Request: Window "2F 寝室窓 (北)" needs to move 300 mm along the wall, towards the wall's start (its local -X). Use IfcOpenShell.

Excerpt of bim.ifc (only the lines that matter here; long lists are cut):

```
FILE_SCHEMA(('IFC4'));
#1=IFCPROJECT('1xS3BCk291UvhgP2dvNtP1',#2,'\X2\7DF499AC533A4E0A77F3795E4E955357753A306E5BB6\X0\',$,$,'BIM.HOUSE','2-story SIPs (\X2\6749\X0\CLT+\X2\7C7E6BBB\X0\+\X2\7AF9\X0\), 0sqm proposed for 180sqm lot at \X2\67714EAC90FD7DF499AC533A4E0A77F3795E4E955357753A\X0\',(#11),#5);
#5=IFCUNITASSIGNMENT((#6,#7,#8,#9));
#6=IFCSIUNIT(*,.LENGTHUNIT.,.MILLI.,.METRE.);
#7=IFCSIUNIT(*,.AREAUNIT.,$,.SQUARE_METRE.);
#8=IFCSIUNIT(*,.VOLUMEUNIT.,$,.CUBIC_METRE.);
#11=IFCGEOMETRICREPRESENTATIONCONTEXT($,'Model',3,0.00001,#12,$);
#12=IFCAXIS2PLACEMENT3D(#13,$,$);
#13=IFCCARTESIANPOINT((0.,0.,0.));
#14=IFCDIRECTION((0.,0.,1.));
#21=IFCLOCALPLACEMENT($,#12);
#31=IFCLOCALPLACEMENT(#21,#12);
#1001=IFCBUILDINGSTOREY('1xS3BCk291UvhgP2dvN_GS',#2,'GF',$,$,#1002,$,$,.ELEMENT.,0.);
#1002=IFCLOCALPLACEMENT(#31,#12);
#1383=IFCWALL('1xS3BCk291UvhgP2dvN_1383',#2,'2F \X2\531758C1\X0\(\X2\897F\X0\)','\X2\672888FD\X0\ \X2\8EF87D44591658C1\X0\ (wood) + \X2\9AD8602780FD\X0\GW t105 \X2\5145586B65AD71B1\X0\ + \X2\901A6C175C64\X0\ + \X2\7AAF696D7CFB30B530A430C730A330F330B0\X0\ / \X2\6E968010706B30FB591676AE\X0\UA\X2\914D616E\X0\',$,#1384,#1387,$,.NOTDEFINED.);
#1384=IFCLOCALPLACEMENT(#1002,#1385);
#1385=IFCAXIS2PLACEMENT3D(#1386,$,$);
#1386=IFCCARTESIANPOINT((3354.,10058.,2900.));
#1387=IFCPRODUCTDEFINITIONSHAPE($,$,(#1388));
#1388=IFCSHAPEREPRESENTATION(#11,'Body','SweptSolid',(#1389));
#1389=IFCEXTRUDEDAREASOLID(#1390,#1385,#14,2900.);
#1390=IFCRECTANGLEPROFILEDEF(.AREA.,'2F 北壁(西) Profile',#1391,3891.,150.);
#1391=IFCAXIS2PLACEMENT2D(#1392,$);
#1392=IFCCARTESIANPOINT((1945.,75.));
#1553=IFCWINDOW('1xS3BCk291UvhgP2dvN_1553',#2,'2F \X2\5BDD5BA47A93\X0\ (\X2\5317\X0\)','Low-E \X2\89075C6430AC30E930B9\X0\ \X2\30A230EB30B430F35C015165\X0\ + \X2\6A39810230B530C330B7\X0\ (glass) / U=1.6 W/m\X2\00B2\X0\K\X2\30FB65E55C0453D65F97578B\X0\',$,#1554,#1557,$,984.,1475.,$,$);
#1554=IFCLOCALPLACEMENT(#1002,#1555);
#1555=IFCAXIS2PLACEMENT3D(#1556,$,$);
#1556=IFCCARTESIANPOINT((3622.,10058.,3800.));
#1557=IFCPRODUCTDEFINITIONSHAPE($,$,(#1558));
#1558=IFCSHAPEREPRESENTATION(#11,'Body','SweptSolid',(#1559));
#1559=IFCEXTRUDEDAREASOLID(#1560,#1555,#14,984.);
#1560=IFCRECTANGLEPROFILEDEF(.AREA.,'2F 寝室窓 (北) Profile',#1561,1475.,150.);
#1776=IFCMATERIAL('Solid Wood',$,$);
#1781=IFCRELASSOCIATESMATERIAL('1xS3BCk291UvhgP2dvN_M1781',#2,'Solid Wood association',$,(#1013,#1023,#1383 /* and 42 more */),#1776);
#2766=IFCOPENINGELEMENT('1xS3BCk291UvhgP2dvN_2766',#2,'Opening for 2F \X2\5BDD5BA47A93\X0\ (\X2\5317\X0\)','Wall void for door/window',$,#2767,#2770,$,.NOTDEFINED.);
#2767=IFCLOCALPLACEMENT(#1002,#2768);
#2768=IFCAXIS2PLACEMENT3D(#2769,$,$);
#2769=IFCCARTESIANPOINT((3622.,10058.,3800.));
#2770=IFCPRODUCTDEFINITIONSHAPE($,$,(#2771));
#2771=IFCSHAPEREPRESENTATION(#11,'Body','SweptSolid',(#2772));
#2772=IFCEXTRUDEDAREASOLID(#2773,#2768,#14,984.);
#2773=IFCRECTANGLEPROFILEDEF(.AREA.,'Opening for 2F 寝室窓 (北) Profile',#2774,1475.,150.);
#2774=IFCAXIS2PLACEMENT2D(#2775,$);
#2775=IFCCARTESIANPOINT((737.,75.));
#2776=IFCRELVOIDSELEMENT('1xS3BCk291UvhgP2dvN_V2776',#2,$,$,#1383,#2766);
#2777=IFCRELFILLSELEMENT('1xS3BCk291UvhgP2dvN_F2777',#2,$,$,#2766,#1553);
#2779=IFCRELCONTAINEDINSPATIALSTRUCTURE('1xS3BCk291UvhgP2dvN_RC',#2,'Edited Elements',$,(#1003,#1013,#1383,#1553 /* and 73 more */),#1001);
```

```python
import ifcopenshell
import ifcopenshell.api.geometry
import ifcopenshell.util.placement

model = ifcopenshell.open("bim.ifc")

window = model.by_id(1553)
opening = window.FillsVoids[0].RelatingOpeningElement
wall = opening.VoidsElements[0].RelatingBuildingElement

wall_matrix = ifcopenshell.util.placement.get_local_placement(wall.ObjectPlacement)
shift = wall_matrix[:3, 0] * -300.0
before = ifcopenshell.util.placement.get_local_placement(window.ObjectPlacement)[:3, 3].copy()

# The window is not placed relative to its opening, so move both.
for product in (opening, window):
    matrix = ifcopenshell.util.placement.get_local_placement(product.ObjectPlacement)
    matrix[:3, 3] += shift
    ifcopenshell.api.geometry.edit_object_placement(model, product=product, matrix=matrix, is_si=False)

after = ifcopenshell.util.placement.get_local_placement(window.ObjectPlacement)[:3, 3]
print("window moved by", (after - before).round(3) + 0.0)

model.write("bim_v2.ifc")
```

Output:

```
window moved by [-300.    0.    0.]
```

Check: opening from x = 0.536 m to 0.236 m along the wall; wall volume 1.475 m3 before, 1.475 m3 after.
